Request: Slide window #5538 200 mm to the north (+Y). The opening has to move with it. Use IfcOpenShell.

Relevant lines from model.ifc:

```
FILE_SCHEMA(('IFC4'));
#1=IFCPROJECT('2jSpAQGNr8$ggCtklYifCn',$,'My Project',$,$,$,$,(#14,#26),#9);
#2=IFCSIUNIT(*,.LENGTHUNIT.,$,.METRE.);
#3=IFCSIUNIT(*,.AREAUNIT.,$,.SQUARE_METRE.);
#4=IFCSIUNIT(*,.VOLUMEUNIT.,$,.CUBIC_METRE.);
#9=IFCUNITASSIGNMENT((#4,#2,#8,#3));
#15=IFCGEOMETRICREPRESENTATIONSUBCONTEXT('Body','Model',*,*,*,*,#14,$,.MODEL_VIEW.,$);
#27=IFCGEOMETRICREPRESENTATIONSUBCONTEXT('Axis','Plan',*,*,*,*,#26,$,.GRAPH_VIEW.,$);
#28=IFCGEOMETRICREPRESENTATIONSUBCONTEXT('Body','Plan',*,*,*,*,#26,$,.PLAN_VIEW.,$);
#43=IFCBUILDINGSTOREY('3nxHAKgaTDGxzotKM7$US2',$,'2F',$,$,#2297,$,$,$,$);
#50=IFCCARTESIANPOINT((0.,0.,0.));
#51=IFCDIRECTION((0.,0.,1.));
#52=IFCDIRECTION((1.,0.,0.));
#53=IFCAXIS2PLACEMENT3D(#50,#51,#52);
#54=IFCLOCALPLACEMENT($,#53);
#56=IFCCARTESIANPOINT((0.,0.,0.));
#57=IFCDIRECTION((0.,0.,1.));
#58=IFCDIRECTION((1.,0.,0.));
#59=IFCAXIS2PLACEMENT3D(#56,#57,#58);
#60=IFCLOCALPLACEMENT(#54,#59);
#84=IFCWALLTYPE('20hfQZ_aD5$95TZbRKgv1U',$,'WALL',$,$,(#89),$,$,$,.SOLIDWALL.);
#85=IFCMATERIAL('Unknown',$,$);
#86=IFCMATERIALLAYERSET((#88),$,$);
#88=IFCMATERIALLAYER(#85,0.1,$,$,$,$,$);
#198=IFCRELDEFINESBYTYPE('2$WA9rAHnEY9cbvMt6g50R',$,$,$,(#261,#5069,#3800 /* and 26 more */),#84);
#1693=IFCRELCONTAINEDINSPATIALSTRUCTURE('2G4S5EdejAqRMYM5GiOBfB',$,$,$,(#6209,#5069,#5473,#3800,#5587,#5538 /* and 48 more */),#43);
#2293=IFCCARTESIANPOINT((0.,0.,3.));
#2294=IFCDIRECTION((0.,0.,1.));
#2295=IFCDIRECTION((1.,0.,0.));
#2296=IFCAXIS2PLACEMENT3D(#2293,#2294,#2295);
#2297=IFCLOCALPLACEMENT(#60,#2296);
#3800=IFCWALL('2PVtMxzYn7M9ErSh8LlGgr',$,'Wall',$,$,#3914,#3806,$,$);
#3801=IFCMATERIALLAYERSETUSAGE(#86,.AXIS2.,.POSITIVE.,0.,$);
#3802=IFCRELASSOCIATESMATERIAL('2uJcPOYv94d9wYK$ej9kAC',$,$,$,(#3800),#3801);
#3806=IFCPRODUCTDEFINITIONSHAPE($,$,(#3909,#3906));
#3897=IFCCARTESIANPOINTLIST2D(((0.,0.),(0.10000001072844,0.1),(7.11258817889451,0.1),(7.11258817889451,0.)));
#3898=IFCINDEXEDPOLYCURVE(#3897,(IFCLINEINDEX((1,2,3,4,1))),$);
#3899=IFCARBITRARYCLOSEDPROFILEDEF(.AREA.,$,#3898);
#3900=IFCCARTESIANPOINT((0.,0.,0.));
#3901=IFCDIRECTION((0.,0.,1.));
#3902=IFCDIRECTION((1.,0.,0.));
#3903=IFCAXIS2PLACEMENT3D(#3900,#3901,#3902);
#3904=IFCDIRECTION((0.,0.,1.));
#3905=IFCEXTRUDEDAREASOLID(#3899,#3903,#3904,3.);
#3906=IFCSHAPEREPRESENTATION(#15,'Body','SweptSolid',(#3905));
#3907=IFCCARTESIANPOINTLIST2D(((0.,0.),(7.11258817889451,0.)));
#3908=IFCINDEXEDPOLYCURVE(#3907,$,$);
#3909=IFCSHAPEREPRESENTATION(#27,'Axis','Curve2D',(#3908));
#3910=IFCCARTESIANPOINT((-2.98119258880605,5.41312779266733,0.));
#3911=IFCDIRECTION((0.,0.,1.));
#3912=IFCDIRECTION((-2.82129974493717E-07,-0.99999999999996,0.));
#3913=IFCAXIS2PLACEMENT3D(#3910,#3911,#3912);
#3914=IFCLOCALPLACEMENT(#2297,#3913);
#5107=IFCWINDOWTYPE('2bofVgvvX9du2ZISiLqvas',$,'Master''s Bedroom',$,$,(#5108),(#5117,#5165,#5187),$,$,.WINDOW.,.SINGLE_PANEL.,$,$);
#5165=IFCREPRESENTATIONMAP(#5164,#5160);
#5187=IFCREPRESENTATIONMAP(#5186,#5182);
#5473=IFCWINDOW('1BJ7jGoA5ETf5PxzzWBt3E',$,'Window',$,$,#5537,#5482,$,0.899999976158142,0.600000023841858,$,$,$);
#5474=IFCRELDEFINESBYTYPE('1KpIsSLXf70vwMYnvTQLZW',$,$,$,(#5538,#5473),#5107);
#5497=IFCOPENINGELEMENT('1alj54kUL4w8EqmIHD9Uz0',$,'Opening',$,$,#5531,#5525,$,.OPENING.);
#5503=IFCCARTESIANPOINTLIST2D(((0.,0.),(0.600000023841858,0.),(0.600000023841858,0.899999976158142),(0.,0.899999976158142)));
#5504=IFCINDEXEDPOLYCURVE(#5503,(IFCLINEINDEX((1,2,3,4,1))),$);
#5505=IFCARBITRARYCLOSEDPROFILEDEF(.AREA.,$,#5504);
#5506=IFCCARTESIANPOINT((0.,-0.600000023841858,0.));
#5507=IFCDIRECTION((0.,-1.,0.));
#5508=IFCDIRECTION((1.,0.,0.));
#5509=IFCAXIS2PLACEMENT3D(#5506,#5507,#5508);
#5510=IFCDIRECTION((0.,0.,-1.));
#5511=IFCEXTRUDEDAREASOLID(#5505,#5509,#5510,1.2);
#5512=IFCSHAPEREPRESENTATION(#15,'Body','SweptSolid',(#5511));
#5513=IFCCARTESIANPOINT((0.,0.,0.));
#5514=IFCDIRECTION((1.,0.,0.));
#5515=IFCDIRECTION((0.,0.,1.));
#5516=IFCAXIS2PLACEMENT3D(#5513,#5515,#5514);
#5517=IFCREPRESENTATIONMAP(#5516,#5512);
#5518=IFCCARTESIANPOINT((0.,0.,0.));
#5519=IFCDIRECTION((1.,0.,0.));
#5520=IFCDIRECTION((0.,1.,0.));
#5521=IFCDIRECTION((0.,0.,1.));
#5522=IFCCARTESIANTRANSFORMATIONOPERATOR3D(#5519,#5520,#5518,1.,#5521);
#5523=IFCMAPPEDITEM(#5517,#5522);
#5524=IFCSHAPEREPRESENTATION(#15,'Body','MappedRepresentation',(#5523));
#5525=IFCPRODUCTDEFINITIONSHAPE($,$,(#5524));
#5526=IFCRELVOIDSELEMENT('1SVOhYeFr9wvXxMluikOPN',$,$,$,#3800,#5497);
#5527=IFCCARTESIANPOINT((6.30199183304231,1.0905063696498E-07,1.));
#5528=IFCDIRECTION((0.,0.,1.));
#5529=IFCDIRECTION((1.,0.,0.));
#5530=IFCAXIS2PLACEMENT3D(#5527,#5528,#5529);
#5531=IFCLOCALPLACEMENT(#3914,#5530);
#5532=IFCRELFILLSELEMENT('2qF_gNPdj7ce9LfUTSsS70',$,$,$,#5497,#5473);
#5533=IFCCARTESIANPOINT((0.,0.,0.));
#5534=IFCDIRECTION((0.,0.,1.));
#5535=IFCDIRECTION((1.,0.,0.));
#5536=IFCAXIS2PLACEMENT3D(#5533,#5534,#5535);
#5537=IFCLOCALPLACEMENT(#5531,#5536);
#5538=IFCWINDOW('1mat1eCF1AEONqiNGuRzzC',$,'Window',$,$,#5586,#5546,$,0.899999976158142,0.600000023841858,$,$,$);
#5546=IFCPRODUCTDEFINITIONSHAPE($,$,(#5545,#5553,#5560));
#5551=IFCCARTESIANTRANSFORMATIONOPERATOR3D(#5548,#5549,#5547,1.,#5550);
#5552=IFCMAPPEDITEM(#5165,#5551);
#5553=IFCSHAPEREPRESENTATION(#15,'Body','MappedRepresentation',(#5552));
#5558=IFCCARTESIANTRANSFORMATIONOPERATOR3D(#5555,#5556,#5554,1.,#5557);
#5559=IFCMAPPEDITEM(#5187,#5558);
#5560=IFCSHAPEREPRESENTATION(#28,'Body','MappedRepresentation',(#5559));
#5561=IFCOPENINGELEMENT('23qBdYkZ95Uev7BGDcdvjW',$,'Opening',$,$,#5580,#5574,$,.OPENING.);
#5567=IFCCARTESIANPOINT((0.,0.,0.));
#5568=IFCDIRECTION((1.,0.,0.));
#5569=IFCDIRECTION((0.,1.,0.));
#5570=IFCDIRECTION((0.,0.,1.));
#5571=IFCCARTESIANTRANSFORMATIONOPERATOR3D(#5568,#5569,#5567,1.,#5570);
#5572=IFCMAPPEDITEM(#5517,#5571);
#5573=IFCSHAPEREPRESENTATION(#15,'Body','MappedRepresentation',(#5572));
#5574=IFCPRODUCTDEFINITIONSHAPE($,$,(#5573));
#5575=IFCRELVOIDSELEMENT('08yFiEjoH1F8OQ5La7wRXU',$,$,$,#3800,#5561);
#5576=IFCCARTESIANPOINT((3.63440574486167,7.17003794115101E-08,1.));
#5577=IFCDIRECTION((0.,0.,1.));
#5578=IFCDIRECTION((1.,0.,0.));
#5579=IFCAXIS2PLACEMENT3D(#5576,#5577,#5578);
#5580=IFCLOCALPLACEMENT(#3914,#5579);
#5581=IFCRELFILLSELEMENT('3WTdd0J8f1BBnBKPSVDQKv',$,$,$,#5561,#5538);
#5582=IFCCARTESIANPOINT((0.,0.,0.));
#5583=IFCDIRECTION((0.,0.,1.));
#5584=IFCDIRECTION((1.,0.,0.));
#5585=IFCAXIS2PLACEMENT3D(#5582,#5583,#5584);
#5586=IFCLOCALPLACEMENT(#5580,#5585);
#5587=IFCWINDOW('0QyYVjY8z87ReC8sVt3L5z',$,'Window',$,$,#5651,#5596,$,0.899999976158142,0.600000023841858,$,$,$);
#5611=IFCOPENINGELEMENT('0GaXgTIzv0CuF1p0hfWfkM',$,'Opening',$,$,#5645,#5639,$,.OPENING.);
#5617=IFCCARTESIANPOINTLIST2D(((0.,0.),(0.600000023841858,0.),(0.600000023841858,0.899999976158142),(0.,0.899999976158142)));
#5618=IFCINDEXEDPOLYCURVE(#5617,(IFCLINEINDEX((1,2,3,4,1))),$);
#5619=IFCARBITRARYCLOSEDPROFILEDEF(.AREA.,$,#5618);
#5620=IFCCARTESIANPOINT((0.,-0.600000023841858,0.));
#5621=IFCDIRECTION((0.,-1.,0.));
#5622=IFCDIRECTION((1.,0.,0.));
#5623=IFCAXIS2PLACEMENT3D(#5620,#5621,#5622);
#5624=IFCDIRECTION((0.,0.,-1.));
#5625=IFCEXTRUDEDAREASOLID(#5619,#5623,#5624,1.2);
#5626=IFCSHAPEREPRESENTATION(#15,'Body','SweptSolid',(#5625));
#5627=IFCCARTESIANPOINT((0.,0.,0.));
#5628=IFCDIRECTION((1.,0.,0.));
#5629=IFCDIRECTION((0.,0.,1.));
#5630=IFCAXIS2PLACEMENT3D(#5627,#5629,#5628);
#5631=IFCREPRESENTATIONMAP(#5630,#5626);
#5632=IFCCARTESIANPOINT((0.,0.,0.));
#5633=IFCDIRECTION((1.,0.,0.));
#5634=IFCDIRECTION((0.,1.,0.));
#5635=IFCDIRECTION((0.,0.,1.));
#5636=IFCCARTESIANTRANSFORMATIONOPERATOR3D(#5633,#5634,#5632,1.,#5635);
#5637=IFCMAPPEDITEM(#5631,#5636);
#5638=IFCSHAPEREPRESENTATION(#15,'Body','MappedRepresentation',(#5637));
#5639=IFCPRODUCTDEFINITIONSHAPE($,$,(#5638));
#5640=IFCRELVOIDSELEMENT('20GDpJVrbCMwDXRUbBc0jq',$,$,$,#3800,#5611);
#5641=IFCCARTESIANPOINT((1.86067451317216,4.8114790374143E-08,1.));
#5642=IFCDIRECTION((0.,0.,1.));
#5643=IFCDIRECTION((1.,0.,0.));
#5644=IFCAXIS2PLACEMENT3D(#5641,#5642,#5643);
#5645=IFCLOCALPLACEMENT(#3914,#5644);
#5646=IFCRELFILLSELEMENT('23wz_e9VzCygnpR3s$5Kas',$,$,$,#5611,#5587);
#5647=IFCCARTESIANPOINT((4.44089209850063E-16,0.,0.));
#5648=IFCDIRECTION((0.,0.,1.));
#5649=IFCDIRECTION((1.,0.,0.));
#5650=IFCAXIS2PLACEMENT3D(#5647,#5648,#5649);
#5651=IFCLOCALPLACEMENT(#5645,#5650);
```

```python
import ifcopenshell
import ifcopenshell.api.geometry
import ifcopenshell.util.placement
import ifcopenshell.util.unit

model = ifcopenshell.open("model.ifc")
unit_scale = ifcopenshell.util.unit.calculate_unit_scale(model)

window = model.by_id(5538)
opening = window.FillsVoids[0].RelatingOpeningElement
wall = opening.VoidsElements[0].RelatingBuildingElement

wall_matrix = ifcopenshell.util.placement.get_local_placement(wall.ObjectPlacement)
shift = wall_matrix[:3, 0] * -0.2 / unit_scale
before = ifcopenshell.util.placement.get_local_placement(window.ObjectPlacement)[:3, 3].copy()

# The window is placed relative to its opening, so it follows when the opening moves.
matrix = ifcopenshell.util.placement.get_local_placement(opening.ObjectPlacement)
matrix[:3, 3] += shift
ifcopenshell.api.geometry.edit_object_placement(
    model, product=opening, matrix=matrix, is_si=False, should_transform_children=True
)

after = ifcopenshell.util.placement.get_local_placement(window.ObjectPlacement)[:3, 3]
print("window moved by", (after - before).round(3) + 0.0)

model.write("model_v2.ifc")
```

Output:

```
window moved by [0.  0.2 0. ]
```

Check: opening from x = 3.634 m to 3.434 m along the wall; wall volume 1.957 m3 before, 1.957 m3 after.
